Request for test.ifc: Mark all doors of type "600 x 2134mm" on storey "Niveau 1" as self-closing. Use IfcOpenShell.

First a look at what the model holds.

```python
import ifcopenshell
import ifcopenshell.util.element

model = ifcopenshell.open("test.ifc")
print(model.schema)
storey = next(s for s in model.by_type("IfcBuildingStorey") if s.Name == "Niveau 1")
doors = [e for e in ifcopenshell.util.element.get_decomposition(storey) if e.is_a("IfcDoor")]
seen = {}
for e in doors:
    element_type = ifcopenshell.util.element.get_type(e)
    key = (element_type.Name if element_type != e and element_type else None, ifcopenshell.util.element.get_pset(e, "Pset_DoorCommon", "SelfClosing"))
    seen[key] = seen.get(key, 0) + 1
for (name, value), count in sorted(seen.items(), key=str):
    print(count, "x", name, "|", value)
```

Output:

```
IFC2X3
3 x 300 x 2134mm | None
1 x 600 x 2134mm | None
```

```python
import ifcopenshell
import ifcopenshell.api.pset
import ifcopenshell.util.element

model = ifcopenshell.open("test.ifc")

storey = next(s for s in model.by_type("IfcBuildingStorey") if s.Name == "Niveau 1")
doors = [e for e in ifcopenshell.util.element.get_decomposition(storey) if e.is_a("IfcDoor")]

count = 0
for e in doors:
    element_type = ifcopenshell.util.element.get_type(e)
    if element_type in (None, e) or element_type.Name != "600 x 2134mm":
        continue
    # add_pset returns the element's existing set when there is one.
    pset = ifcopenshell.api.pset.add_pset(model, product=e, name="Pset_DoorCommon")
    ifcopenshell.api.pset.edit_pset(model, pset=pset, properties={"SelfClosing": True})
    count += 1

print(count, "doors updated")

model.write("test_edited.ifc")
```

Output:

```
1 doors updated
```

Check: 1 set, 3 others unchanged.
